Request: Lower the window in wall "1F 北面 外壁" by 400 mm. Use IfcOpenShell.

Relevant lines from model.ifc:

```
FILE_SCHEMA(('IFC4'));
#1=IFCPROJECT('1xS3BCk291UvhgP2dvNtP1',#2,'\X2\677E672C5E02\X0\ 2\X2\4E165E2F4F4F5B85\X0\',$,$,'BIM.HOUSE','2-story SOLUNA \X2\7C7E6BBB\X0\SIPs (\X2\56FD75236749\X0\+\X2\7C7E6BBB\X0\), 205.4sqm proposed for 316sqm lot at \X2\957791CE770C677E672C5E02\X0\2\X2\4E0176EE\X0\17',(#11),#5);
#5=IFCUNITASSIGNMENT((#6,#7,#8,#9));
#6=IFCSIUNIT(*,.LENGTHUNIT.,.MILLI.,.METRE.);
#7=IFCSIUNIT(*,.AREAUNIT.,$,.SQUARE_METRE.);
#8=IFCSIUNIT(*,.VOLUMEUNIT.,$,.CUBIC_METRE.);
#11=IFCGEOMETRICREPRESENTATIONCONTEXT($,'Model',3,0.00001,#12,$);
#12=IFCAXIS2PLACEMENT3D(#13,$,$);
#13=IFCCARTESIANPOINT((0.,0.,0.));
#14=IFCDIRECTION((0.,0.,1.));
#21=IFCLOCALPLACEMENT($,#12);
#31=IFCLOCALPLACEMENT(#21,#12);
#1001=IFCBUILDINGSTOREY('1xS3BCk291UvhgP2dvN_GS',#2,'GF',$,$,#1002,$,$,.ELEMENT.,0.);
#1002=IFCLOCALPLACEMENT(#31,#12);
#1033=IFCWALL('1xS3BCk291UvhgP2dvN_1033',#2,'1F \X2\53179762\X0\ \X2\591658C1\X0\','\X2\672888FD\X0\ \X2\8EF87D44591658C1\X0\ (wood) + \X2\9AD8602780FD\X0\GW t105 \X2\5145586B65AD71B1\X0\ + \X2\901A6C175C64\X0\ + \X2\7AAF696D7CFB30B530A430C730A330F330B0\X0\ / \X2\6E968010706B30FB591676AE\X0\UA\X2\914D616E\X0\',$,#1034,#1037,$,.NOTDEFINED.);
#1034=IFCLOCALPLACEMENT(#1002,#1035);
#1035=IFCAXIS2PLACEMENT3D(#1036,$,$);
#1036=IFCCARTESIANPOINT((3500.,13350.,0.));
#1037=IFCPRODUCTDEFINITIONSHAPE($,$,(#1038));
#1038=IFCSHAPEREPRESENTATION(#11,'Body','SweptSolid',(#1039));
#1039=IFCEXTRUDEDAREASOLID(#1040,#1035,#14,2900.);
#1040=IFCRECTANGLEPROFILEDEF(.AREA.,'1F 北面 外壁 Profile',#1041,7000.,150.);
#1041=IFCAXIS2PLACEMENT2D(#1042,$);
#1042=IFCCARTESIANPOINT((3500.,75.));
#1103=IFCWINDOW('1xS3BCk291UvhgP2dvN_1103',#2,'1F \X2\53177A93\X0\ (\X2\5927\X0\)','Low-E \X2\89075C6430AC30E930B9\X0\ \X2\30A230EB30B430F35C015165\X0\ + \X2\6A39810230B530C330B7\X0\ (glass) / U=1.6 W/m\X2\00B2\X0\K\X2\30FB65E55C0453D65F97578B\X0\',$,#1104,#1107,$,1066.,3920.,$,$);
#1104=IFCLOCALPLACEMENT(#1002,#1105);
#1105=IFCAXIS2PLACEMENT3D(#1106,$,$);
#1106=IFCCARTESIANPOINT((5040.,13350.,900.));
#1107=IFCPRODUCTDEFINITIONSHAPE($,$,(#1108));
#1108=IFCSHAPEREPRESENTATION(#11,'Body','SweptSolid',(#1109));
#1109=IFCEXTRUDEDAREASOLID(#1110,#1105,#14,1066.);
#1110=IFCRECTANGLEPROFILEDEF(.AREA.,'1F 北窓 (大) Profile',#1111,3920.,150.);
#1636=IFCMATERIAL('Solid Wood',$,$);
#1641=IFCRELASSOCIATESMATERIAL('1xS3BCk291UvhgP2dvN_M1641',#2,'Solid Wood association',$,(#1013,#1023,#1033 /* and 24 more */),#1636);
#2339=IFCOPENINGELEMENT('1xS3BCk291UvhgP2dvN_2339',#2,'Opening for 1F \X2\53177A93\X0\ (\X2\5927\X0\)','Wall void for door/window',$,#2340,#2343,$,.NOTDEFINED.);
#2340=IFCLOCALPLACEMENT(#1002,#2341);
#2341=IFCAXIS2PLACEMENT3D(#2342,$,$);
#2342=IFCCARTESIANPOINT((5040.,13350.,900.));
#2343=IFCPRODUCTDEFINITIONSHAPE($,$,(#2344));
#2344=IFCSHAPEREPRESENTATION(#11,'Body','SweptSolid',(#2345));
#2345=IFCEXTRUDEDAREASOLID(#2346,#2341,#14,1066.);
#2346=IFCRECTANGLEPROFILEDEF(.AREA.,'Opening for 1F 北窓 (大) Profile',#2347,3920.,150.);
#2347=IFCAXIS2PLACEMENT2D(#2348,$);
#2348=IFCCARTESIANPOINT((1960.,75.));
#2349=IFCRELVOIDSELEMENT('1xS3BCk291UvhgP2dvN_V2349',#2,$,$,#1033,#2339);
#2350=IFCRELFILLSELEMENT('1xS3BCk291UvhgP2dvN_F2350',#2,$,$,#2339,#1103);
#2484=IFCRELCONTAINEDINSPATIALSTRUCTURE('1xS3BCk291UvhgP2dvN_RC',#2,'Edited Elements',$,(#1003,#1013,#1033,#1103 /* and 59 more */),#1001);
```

```python
import numpy as np
import ifcopenshell
import ifcopenshell.api.geometry
import ifcopenshell.util.placement
import ifcopenshell.util.unit

model = ifcopenshell.open("model.ifc")
unit_scale = ifcopenshell.util.unit.calculate_unit_scale(model)

window = model.by_guid("1xS3BCk291UvhgP2dvN_1103")
opening = window.FillsVoids[0].RelatingOpeningElement
dz = -400.0

shift = np.array([0.0, 0.0, dz])
# The window is not placed relative to its opening, so move both.
for product in (opening, window):
    matrix = ifcopenshell.util.placement.get_local_placement(product.ObjectPlacement)
    matrix[:3, 3] += shift
    ifcopenshell.api.geometry.edit_object_placement(model, product=product, matrix=matrix, is_si=False)

print(f"moved by {dz * unit_scale:+.3f} m")

model.write("model_edited.ifc")
```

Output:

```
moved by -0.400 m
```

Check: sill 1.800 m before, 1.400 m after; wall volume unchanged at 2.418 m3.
